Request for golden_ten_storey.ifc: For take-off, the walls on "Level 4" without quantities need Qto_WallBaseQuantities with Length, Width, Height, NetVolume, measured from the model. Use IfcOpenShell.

First a look at what the model holds.

```python
import ifcopenshell
import ifcopenshell.util.element
import ifcopenshell.util.unit

model = ifcopenshell.open("golden_ten_storey.ifc")
print(model.schema)
for unit_type in ("LENGTHUNIT", "AREAUNIT", "VOLUMEUNIT"):
    print(unit_type, ifcopenshell.util.unit.calculate_unit_scale(model, unit_type))
storey = next(s for s in model.by_type("IfcBuildingStorey") if s.Name == "Level 4")
walls = [e for e in ifcopenshell.util.element.get_decomposition(storey) if e.is_a("IfcWall")]
for e in sorted(walls, key=lambda e: e.id()):
    print(e.id(), e.is_a(), e.Name, list(ifcopenshell.util.element.get_psets(e, qtos_only=True)), sep=" | ")
```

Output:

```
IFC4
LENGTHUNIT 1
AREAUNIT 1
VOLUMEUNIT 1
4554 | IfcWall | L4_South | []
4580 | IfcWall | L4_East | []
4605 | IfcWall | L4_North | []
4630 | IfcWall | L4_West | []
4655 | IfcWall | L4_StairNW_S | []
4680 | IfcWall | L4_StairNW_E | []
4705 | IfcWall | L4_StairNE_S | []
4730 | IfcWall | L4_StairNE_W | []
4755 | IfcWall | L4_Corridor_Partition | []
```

```python
import ifcopenshell
import ifcopenshell.api.pset
import ifcopenshell.geom
import ifcopenshell.util.element
import ifcopenshell.util.shape
import ifcopenshell.util.unit

model = ifcopenshell.open("golden_ten_storey.ifc")
unit_scale = ifcopenshell.util.unit.calculate_unit_scale(model)
volume_scale = ifcopenshell.util.unit.calculate_unit_scale(model, "VOLUMEUNIT")
settings = ifcopenshell.geom.settings()

storey = next(s for s in model.by_type("IfcBuildingStorey") if s.Name == "Level 4")
walls = [e for e in ifcopenshell.util.element.get_decomposition(storey) if e.is_a("IfcWall")]

for e in sorted(walls, key=lambda e: e.id()):
    if ifcopenshell.util.element.get_psets(e, qtos_only=True, should_inherit=False):
        continue
    # Geometry comes back in metres, in the element's own axes.
    shape = ifcopenshell.geom.create_shape(settings, e)
    values = {
        "Length": ifcopenshell.util.shape.get_x(shape.geometry) / unit_scale,
        "Width": ifcopenshell.util.shape.get_y(shape.geometry) / unit_scale,
        "Height": ifcopenshell.util.shape.get_z(shape.geometry) / unit_scale,
        "NetVolume": ifcopenshell.util.shape.get_volume(shape.geometry) / volume_scale,
    }
    qto = ifcopenshell.api.pset.add_qto(model, product=e, name="Qto_WallBaseQuantities")
    ifcopenshell.api.pset.edit_qto(model, qto=qto, properties=values)
    print(e.id(), {k: round(v, 3) for k, v in values.items()})

model.write("golden_ten_storey_v2.ifc")
```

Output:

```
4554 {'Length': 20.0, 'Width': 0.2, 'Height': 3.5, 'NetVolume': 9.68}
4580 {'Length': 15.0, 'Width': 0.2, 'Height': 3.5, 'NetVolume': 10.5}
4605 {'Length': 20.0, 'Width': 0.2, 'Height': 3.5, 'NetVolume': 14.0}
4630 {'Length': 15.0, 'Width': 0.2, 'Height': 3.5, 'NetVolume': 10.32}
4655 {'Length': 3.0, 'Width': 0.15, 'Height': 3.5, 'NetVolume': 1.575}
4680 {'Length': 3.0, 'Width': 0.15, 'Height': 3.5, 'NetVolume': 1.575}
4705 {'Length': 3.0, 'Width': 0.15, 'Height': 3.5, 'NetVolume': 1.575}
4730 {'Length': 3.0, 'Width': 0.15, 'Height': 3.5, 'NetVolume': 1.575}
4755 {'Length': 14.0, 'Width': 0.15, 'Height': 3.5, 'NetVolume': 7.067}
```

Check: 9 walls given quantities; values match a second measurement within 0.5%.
